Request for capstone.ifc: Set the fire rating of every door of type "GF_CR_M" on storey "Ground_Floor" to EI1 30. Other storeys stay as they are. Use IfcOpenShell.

First a look at what the model holds.

```python
import ifcopenshell
import ifcopenshell.util.element

model = ifcopenshell.open("capstone.ifc")
print(model.schema)
storey = next(s for s in model.by_type("IfcBuildingStorey") if s.Name == "Ground_Floor")
doors = [e for e in ifcopenshell.util.element.get_decomposition(storey) if e.is_a("IfcDoor")]
seen = {}
for e in doors:
    element_type = ifcopenshell.util.element.get_type(e)
    key = (element_type.Name if element_type != e and element_type else None, ifcopenshell.util.element.get_pset(e, "Pset_DoorCommon", "FireRating"))
    seen[key] = seen.get(key, 0) + 1
for (name, value), count in sorted(seen.items(), key=str):
    print(count, "x", name, "|", value)
```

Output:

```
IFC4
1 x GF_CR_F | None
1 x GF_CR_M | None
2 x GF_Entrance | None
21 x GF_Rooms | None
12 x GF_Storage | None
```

```python
import ifcopenshell
import ifcopenshell.api.pset
import ifcopenshell.util.element

model = ifcopenshell.open("capstone.ifc")

storey = next(s for s in model.by_type("IfcBuildingStorey") if s.Name == "Ground_Floor")
doors = [e for e in ifcopenshell.util.element.get_decomposition(storey) if e.is_a("IfcDoor")]

count = 0
for e in doors:
    element_type = ifcopenshell.util.element.get_type(e)
    if element_type in (None, e) or element_type.Name != "GF_CR_M":
        continue
    # add_pset returns the element's existing set when there is one.
    pset = ifcopenshell.api.pset.add_pset(model, product=e, name="Pset_DoorCommon")
    ifcopenshell.api.pset.edit_pset(model, pset=pset, properties={"FireRating": "EI1 30"})
    count += 1

print(count, "doors updated")

model.write("capstone_edited.ifc")
```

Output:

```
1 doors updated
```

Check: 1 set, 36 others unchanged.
